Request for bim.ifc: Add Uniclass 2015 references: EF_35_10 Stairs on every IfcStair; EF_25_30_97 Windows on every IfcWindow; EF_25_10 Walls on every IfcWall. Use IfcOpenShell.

First a look at what the model holds.

```python
import ifcopenshell

model = ifcopenshell.open("bim.ifc")
print(model.schema)
print("classifications:", [c.Name for c in model.by_type("IfcClassification")])
for ifc_class in ("IfcDoor", "IfcRoof", "IfcStair", "IfcWall", "IfcWindow"):
    print(ifc_class, len(model.by_type(ifc_class)))
```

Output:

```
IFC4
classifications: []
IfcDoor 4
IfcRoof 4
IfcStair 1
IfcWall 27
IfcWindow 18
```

```python
import ifcopenshell
import ifcopenshell.api.classification

model = ifcopenshell.open("bim.ifc")

system = ifcopenshell.api.classification.add_classification(model, classification="Uniclass 2015")

codes = {
    "IfcStair": ("EF_35_10", "Stairs"),
    "IfcWindow": ("EF_25_30_97", "Windows"),
    "IfcWall": ("EF_25_10", "Walls"),
}
for ifc_class, (code, name) in codes.items():
    products = model.by_type(ifc_class)
    ifcopenshell.api.classification.add_reference(
        model, products=products, classification=system, identification=code, name=name
    )
    print(code, len(products))

model.write("bim-out.ifc")
```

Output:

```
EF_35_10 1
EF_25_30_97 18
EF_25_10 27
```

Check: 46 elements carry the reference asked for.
